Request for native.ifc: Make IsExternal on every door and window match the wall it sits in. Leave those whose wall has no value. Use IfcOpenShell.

First a look at what the model holds.

```python
import ifcopenshell
import ifcopenshell.util.element

model = ifcopenshell.open("native.ifc")
print(model.schema)
seen = {}
for e in model.by_type("IfcDoor") + model.by_type("IfcWindow"):
    if not e.FillsVoids:
        continue
    host = e.FillsVoids[0].RelatingOpeningElement.VoidsElements[0].RelatingBuildingElement
    own = ifcopenshell.util.element.get_pset(e, f"Pset_{e.is_a()[3:].removesuffix('StandardCase')}Common", "IsExternal")
    wall = ifcopenshell.util.element.get_pset(host, "Pset_WallCommon", "IsExternal")
    seen[e.is_a(), own, wall] = seen.get((e.is_a(), own, wall), 0) + 1
for (cls, own, wall), count in sorted(seen.items(), key=str):
    print(count, cls, "IsExternal:", own, "| host wall:", wall)
```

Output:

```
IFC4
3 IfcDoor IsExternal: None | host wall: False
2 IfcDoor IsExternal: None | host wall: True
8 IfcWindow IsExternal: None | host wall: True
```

```python
import ifcopenshell
import ifcopenshell.api.pset
import ifcopenshell.util.element

model = ifcopenshell.open("native.ifc")

count = 0
for ifc_class, pset_name in (("IfcDoor", "Pset_DoorCommon"), ("IfcWindow", "Pset_WindowCommon")):
    for e in model.by_type(ifc_class):
        if not e.FillsVoids:
            continue
        host = e.FillsVoids[0].RelatingOpeningElement.VoidsElements[0].RelatingBuildingElement
        external = ifcopenshell.util.element.get_pset(host, "Pset_WallCommon", "IsExternal")
        if external is None or ifcopenshell.util.element.get_pset(e, pset_name, "IsExternal") == external:
            continue
        found = ifcopenshell.util.element.get_pset(e, pset_name, should_inherit=False)
        if found:
            pset = model.by_id(found["id"])
            if len(ifcopenshell.util.element.get_elements_by_pset(pset)) > 1:
                pset = ifcopenshell.api.pset.unshare_pset(model, products=[e], pset=pset)[0]
        else:
            pset = ifcopenshell.api.pset.add_pset(model, product=e, name=pset_name)
        ifcopenshell.api.pset.edit_pset(model, pset=pset, properties={"IsExternal": external})
        count += 1

print(count, "updated")

model.write("native_updated.ifc")
```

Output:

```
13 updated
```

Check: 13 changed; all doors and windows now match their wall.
